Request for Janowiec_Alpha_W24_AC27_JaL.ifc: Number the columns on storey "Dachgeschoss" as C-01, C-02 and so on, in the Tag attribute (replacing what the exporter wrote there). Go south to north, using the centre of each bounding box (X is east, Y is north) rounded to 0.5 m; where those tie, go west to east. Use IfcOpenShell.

First a look at what the model holds.

```python
import ifcopenshell
import ifcopenshell.util.element
import ifcopenshell.util.placement

model = ifcopenshell.open("Janowiec_Alpha_W24_AC27_JaL.ifc")
print(model.schema)
storey = next(s for s in model.by_type("IfcBuildingStorey") if s.Name == "Dachgeschoss")
columns = [e for e in ifcopenshell.util.element.get_decomposition(storey) if e.is_a("IfcColumn")]
for e in sorted(columns, key=lambda e: e.id()):
    origin = ifcopenshell.util.placement.get_local_placement(e.ObjectPlacement)[:3, 3]
    print(e.id(), e.Tag, e.Name, origin.round(2) + 0.0, sep=" | ")
```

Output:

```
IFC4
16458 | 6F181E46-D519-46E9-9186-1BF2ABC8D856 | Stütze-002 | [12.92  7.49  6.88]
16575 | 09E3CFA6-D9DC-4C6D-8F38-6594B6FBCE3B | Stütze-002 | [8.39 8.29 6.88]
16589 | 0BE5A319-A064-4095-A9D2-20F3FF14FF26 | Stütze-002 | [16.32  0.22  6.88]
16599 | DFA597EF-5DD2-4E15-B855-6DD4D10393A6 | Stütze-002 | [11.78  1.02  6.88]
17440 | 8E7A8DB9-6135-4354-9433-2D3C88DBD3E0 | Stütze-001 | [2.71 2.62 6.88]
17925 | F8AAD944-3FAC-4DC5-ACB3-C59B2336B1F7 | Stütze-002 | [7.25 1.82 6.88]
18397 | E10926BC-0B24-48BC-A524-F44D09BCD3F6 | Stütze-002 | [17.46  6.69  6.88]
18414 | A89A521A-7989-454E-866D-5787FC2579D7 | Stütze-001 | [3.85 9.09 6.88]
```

```python
import ifcopenshell
import ifcopenshell.geom
import ifcopenshell.util.element
import ifcopenshell.util.shape

model = ifcopenshell.open("Janowiec_Alpha_W24_AC27_JaL.ifc")
settings = ifcopenshell.geom.settings()
settings.set("use-world-coords", True)


def centre(element):
    shape = ifcopenshell.geom.create_shape(settings, element)
    return ifcopenshell.util.shape.get_bbox_centroid(shape.geometry)


storey = next(s for s in model.by_type("IfcBuildingStorey") if s.Name == "Dachgeschoss")
columns = [e for e in ifcopenshell.util.element.get_decomposition(storey) if e.is_a("IfcColumn")]

# Insertion points can sit at a corner or the storey origin, so sort by the geometry (in metres).
centres = {e: centre(e) for e in columns}
columns.sort(key=lambda e: (round(centres[e][1] / 0.5), centres[e][0]))

for i, e in enumerate(columns, start=1):
    number = f"C-{i:02d}"
    e.Tag = number
    print(e.id(), number)

model.write("Janowiec_Alpha_W24_AC27_JaL_edited.ifc")
```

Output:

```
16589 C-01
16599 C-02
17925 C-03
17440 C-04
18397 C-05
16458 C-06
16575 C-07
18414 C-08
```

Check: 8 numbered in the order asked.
